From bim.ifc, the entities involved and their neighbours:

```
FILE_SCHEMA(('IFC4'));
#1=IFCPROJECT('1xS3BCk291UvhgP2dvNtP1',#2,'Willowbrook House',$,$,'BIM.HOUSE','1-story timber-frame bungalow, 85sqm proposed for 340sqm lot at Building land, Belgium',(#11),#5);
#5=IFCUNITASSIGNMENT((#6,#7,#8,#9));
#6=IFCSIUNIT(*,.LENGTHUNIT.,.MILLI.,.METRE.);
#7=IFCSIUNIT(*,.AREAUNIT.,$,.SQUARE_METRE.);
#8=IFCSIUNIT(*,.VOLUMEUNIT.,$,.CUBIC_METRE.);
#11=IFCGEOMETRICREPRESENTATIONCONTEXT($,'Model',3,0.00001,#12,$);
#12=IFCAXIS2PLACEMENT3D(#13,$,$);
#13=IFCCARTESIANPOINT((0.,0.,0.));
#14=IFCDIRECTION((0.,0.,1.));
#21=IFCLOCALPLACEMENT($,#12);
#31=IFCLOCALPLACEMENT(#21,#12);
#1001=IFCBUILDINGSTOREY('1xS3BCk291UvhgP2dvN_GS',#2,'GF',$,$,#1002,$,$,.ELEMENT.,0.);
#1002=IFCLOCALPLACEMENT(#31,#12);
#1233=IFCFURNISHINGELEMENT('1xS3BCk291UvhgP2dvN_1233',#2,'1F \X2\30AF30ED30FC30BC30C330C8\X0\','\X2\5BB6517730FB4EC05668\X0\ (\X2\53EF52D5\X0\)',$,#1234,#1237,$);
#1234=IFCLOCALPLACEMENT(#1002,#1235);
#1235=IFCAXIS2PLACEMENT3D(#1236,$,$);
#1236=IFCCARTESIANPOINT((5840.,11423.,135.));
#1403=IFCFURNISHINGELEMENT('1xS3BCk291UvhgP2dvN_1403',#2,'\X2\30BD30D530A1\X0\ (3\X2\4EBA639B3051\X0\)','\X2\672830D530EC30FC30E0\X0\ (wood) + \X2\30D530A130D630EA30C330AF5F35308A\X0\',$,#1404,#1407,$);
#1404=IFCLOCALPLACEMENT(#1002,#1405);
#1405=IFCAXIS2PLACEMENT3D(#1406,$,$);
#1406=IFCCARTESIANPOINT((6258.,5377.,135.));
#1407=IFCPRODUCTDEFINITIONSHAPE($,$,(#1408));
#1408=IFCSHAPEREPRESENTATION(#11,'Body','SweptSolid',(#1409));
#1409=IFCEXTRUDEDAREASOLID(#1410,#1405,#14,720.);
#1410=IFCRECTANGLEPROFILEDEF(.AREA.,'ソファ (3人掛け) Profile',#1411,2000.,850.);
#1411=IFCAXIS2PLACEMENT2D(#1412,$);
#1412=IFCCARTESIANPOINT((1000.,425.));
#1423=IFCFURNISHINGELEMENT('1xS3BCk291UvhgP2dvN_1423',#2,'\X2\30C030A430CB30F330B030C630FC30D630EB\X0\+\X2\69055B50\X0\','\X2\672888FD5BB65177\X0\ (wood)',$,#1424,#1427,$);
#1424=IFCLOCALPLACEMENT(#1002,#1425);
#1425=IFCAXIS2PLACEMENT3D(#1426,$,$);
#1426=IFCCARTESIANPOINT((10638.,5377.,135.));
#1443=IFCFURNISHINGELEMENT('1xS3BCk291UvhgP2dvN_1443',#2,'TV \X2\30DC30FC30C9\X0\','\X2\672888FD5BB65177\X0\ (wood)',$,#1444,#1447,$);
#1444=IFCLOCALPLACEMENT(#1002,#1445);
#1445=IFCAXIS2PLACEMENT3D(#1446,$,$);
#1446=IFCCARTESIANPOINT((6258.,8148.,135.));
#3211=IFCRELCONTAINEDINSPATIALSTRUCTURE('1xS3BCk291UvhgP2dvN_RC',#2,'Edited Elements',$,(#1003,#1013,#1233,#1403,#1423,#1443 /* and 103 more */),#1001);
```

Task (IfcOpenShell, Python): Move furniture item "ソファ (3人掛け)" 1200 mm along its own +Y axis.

```python
import ifcopenshell
import ifcopenshell.api.geometry
import ifcopenshell.util.placement
import ifcopenshell.util.unit

model = ifcopenshell.open("bim.ifc")
unit_scale = ifcopenshell.util.unit.calculate_unit_scale(model)

item = model.by_guid("1xS3BCk291UvhgP2dvN_1403")
matrix = ifcopenshell.util.placement.get_local_placement(item.ObjectPlacement)
matrix[:3, 3] += matrix[:3, 1] * 1.2 / unit_scale
ifcopenshell.api.geometry.edit_object_placement(model, product=item, matrix=matrix, is_si=False)

print(ifcopenshell.util.placement.get_local_placement(item.ObjectPlacement).round(3) + 0.0)

model.write("bim_edited.ifc")
```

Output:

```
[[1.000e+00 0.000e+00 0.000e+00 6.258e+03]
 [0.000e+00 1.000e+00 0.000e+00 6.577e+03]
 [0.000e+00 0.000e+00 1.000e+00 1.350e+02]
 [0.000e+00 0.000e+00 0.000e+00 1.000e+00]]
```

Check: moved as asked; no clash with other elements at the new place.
